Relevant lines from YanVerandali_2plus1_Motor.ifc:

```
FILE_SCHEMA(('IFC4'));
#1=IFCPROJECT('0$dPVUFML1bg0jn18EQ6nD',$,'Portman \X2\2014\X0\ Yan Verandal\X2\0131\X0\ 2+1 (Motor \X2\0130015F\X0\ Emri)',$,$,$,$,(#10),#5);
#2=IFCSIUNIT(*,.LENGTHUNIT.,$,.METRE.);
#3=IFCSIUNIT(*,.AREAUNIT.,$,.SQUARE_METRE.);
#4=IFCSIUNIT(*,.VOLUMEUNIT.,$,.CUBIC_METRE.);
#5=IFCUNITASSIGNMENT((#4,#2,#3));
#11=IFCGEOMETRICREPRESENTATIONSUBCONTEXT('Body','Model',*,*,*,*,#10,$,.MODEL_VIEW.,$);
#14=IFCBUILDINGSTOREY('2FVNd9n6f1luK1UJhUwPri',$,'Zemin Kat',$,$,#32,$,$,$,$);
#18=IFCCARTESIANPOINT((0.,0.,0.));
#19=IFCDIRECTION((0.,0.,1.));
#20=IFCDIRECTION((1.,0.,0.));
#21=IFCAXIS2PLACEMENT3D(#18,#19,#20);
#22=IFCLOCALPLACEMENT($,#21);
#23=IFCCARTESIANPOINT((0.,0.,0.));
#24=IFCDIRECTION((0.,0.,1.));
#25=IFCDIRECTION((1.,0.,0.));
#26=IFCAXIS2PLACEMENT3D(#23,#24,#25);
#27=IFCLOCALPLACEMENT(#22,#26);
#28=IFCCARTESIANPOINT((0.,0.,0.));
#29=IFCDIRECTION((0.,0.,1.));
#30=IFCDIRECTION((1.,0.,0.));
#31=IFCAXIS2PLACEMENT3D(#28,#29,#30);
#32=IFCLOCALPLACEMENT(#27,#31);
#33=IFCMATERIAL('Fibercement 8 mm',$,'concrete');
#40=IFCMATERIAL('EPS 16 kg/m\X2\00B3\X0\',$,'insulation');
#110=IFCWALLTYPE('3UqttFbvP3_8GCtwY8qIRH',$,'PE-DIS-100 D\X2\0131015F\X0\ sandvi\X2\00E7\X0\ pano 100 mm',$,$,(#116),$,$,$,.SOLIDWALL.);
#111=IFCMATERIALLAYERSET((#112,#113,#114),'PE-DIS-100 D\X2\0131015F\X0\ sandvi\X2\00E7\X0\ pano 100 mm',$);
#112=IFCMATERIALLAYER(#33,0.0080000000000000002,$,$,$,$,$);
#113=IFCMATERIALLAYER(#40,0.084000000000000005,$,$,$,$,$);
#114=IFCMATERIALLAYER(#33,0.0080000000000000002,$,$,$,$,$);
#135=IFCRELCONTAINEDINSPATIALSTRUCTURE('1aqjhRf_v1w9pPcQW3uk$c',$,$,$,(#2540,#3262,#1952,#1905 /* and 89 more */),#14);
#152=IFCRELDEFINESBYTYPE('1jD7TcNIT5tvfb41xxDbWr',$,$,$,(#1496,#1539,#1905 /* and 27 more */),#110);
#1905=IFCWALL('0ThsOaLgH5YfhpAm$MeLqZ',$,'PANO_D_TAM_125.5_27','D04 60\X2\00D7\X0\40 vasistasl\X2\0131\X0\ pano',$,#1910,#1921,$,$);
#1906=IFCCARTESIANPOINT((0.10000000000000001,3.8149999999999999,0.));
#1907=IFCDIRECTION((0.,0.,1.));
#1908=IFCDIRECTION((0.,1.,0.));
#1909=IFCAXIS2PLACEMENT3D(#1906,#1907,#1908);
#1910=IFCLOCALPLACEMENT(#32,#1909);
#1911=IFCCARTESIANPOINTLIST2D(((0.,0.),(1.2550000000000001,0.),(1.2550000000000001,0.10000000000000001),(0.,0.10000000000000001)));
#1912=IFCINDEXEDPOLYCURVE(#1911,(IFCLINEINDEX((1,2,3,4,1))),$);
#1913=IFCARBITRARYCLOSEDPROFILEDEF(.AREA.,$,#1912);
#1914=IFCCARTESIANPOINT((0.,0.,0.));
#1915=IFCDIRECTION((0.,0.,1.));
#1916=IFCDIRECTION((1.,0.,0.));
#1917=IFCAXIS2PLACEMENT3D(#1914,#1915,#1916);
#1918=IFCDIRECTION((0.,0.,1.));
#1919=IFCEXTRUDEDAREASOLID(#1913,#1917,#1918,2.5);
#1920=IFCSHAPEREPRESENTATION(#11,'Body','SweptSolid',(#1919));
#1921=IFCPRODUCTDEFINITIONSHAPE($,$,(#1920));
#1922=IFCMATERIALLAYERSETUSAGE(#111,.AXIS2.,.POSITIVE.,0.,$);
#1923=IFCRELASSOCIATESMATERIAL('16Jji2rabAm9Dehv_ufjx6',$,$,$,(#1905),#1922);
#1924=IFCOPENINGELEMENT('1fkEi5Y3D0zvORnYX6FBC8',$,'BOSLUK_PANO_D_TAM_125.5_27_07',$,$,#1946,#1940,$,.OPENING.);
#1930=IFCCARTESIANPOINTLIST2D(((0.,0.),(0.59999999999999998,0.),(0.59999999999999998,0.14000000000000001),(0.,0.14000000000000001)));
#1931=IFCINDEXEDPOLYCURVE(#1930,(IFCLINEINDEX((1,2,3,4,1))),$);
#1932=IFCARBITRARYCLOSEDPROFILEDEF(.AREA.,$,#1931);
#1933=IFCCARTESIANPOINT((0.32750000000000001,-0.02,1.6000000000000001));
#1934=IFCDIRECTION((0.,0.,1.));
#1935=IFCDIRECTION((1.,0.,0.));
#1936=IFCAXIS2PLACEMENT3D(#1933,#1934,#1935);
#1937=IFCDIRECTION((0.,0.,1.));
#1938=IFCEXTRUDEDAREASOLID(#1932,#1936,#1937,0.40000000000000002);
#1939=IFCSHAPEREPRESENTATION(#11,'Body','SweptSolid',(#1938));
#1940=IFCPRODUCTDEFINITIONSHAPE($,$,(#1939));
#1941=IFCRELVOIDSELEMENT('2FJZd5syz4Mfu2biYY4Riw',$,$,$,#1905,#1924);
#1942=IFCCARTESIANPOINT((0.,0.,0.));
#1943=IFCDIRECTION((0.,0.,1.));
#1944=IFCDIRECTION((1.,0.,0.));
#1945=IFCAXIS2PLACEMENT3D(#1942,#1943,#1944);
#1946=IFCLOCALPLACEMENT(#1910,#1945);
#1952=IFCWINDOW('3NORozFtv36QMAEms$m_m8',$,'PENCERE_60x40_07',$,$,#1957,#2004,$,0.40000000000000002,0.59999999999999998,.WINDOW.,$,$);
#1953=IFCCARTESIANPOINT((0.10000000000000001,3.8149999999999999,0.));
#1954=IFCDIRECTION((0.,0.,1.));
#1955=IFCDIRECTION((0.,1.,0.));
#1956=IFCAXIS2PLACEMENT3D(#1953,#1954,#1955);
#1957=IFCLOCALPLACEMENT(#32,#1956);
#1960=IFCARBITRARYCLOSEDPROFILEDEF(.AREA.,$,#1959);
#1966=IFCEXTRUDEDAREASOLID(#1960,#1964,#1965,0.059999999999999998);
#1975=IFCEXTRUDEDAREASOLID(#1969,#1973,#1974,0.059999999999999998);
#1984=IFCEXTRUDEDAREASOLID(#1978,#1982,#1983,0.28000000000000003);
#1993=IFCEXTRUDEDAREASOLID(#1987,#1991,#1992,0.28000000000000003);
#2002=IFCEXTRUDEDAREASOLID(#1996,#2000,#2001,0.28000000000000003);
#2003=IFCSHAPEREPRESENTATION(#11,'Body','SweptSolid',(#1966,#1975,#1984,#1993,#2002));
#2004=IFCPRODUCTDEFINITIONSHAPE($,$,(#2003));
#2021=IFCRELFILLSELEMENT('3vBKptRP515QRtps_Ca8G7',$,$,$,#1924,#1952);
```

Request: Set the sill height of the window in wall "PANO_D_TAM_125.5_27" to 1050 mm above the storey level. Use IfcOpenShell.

```python
import numpy as np
import ifcopenshell
import ifcopenshell.api.geometry
import ifcopenshell.geom
import ifcopenshell.util.element
import ifcopenshell.util.placement
import ifcopenshell.util.shape
import ifcopenshell.util.unit

model = ifcopenshell.open("YanVerandali_2plus1_Motor.ifc")
unit_scale = ifcopenshell.util.unit.calculate_unit_scale(model)

window = model.by_id(1952)
opening = window.FillsVoids[0].RelatingOpeningElement
storey = ifcopenshell.util.element.get_container(window, ifc_class="IfcBuildingStorey")
level = ifcopenshell.util.placement.get_local_placement(storey.ObjectPlacement)[2, 3]

# The opening's origin need not be at the sill, so measure its lowest point.
shape = ifcopenshell.geom.create_shape(ifcopenshell.geom.settings(), opening)
bottom = ifcopenshell.util.shape.get_shape_bottom_elevation(shape, shape.geometry) / unit_scale
dz = level + 1.05 / unit_scale - bottom

shift = np.array([0.0, 0.0, dz])
# The window is not placed relative to its opening, so move both.
for product in (opening, window):
    matrix = ifcopenshell.util.placement.get_local_placement(product.ObjectPlacement)
    matrix[:3, 3] += shift
    ifcopenshell.api.geometry.edit_object_placement(model, product=product, matrix=matrix, is_si=False)

print(f"moved by {dz * unit_scale:+.3f} m")

model.write("YanVerandali_2plus1_Motor-out.ifc")
```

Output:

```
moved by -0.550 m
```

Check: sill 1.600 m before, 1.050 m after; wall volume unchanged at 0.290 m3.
